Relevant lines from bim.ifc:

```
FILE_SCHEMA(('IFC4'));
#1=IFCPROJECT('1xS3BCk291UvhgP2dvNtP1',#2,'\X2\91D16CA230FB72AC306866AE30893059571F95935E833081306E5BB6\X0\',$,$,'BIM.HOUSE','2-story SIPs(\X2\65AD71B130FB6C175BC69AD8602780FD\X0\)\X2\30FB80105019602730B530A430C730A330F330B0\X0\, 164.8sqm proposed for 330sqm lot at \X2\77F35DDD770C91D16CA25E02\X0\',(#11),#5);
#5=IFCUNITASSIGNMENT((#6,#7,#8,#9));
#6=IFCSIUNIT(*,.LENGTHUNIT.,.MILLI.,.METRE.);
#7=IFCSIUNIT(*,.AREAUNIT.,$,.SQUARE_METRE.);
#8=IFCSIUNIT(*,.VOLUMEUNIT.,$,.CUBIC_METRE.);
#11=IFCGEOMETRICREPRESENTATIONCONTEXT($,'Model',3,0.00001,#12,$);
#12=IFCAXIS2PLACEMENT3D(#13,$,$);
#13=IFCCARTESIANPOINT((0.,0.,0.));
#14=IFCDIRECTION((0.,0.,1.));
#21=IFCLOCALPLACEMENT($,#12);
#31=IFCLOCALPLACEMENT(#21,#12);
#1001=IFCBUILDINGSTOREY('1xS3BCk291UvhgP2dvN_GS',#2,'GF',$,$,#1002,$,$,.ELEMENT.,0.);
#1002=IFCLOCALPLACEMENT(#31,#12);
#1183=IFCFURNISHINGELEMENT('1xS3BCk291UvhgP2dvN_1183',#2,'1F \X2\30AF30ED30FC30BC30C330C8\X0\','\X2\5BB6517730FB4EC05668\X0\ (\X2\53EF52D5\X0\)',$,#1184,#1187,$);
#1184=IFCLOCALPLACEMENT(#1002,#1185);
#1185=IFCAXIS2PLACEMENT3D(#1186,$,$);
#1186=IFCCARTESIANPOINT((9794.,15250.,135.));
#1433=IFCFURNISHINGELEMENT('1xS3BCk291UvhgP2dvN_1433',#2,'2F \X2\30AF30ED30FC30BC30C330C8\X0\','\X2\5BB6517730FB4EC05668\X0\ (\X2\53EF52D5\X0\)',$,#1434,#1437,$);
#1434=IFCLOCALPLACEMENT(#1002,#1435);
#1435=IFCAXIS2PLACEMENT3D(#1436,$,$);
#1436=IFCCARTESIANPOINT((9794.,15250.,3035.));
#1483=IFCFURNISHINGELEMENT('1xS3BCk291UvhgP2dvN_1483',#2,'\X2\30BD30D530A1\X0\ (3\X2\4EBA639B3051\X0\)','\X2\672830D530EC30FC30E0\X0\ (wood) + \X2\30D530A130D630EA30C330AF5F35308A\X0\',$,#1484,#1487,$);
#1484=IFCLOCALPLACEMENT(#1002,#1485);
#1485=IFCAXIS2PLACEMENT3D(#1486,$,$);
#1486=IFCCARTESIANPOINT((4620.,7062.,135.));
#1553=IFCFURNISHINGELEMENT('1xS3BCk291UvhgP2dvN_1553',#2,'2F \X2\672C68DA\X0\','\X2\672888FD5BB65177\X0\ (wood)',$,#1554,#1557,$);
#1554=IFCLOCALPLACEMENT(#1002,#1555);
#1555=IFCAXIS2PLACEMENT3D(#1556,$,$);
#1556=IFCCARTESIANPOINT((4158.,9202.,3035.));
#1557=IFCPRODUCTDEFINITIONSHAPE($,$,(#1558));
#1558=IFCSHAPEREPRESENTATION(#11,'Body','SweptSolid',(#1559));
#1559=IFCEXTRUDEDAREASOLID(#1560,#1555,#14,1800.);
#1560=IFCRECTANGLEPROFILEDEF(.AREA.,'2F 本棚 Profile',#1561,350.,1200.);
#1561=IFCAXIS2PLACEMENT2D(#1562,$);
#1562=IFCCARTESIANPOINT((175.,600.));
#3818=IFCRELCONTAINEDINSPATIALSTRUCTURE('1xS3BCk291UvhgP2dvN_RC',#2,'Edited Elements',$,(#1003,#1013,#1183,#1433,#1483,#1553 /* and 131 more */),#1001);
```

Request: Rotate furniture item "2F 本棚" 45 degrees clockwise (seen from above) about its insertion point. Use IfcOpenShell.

```python
import ifcopenshell
import ifcopenshell.api.geometry
import ifcopenshell.util.placement

model = ifcopenshell.open("bim.ifc")

item = model.by_id(1553)
matrix = ifcopenshell.util.placement.get_local_placement(item.ObjectPlacement)
matrix = matrix @ ifcopenshell.util.placement.rotation(-45, "Z")
ifcopenshell.api.geometry.edit_object_placement(model, product=item, matrix=matrix, is_si=False)

print(ifcopenshell.util.placement.get_local_placement(item.ObjectPlacement).round(3) + 0.0)

model.write("bim-out.ifc")
```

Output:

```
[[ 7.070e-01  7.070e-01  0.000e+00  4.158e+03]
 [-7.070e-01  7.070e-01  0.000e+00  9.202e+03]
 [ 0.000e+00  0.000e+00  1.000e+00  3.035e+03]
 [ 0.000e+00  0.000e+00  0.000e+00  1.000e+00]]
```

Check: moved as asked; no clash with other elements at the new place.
